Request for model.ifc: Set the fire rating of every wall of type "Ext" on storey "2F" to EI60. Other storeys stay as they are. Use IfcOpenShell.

First a look at what the model holds.

```python
import ifcopenshell
import ifcopenshell.util.element

model = ifcopenshell.open("model.ifc")
print(model.schema)
storey = next(s for s in model.by_type("IfcBuildingStorey") if s.Name == "2F")
walls = [e for e in ifcopenshell.util.element.get_decomposition(storey) if e.is_a("IfcWall")]
seen = {}
for e in walls:
    element_type = ifcopenshell.util.element.get_type(e)
    key = (element_type.Name if element_type != e and element_type else None, ifcopenshell.util.element.get_pset(e, "Pset_WallCommon", "FireRating"))
    seen[key] = seen.get(key, 0) + 1
for (name, value), count in sorted(seen.items(), key=str):
    print(count, "x", name, "|", value)
```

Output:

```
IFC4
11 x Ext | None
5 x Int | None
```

```python
import ifcopenshell
import ifcopenshell.api.pset
import ifcopenshell.util.element

model = ifcopenshell.open("model.ifc")

storey = next(s for s in model.by_type("IfcBuildingStorey") if s.Name == "2F")
walls = [e for e in ifcopenshell.util.element.get_decomposition(storey) if e.is_a("IfcWall")]

count = 0
for e in walls:
    element_type = ifcopenshell.util.element.get_type(e)
    if element_type in (None, e) or element_type.Name != "Ext":
        continue
    # add_pset returns the element's existing set when there is one.
    pset = ifcopenshell.api.pset.add_pset(model, product=e, name="Pset_WallCommon")
    ifcopenshell.api.pset.edit_pset(model, pset=pset, properties={"FireRating": "EI60"})
    count += 1

print(count, "walls updated")

model.write("model-out.ifc")
```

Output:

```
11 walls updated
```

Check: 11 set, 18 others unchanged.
